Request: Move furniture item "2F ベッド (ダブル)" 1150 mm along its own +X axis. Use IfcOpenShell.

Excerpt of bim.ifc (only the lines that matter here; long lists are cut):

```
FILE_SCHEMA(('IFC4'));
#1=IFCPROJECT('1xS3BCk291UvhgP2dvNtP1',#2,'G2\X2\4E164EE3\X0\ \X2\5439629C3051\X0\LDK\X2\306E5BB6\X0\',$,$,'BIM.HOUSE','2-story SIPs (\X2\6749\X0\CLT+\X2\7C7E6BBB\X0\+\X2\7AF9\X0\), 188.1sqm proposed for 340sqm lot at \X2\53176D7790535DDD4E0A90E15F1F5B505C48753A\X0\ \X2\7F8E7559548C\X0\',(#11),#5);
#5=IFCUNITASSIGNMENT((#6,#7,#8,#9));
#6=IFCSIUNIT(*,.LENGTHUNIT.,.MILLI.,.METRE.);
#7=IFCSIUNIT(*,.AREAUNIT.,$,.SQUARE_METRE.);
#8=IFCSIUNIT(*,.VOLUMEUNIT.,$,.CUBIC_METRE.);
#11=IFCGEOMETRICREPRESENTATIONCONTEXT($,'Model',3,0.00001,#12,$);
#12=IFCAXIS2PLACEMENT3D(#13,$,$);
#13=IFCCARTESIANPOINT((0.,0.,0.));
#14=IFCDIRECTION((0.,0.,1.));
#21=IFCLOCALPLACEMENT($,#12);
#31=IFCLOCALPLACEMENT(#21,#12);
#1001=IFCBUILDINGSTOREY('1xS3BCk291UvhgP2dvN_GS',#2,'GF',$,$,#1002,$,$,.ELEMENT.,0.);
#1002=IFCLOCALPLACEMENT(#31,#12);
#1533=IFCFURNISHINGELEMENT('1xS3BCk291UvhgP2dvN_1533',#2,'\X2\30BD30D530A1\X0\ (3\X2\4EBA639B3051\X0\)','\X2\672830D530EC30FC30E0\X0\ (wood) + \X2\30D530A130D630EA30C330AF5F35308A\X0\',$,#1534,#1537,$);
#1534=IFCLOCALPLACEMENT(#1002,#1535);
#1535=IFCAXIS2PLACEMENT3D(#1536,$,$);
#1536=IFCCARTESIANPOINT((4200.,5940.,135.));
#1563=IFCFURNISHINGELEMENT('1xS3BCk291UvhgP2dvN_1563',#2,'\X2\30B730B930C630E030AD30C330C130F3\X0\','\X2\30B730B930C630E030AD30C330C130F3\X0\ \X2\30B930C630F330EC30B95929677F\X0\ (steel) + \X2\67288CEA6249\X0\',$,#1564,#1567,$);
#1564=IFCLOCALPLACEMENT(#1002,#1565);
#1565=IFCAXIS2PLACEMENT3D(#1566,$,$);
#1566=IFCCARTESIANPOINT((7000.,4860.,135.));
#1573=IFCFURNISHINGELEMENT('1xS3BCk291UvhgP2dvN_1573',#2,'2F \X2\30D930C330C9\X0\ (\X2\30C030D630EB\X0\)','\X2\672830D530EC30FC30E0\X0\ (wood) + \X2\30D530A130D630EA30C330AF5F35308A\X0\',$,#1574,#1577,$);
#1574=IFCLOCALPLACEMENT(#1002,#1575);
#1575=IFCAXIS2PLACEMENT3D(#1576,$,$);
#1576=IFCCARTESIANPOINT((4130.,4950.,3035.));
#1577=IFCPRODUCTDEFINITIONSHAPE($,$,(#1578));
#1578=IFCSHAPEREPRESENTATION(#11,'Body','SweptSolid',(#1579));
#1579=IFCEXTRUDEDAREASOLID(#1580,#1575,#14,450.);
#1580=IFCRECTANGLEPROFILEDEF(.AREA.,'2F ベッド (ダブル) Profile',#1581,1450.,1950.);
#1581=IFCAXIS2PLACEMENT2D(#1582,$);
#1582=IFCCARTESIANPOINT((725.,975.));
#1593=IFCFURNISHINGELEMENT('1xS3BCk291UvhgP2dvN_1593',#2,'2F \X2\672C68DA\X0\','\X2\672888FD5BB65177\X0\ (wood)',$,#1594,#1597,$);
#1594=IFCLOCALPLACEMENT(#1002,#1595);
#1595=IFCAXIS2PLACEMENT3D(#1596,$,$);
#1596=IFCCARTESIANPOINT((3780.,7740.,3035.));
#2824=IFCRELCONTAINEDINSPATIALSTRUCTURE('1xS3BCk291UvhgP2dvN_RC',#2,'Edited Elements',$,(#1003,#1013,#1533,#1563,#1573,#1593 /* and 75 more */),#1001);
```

```python
import ifcopenshell
import ifcopenshell.api.geometry
import ifcopenshell.util.placement
import ifcopenshell.util.unit

model = ifcopenshell.open("bim.ifc")
unit_scale = ifcopenshell.util.unit.calculate_unit_scale(model)

item = model.by_guid("1xS3BCk291UvhgP2dvN_1573")
matrix = ifcopenshell.util.placement.get_local_placement(item.ObjectPlacement)
matrix[:3, 3] += matrix[:3, 0] * 1.15 / unit_scale
ifcopenshell.api.geometry.edit_object_placement(model, product=item, matrix=matrix, is_si=False)

print(ifcopenshell.util.placement.get_local_placement(item.ObjectPlacement).round(3) + 0.0)

model.write("bim-out.ifc")
```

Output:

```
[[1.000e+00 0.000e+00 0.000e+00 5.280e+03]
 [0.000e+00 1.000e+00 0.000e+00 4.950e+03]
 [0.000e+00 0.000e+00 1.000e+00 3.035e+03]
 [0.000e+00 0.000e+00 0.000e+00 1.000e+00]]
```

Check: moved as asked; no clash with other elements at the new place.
